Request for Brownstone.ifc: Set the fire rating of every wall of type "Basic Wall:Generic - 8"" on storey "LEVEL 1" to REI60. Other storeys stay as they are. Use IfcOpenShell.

First a look at what the model holds.

```python
import ifcopenshell
import ifcopenshell.util.element

model = ifcopenshell.open("Brownstone.ifc")
print(model.schema)
storey = next(s for s in model.by_type("IfcBuildingStorey") if s.Name == "LEVEL 1")
walls = [e for e in ifcopenshell.util.element.get_decomposition(storey) if e.is_a("IfcWall")]
seen = {}
for e in walls:
    element_type = ifcopenshell.util.element.get_type(e)
    key = (element_type.Name if element_type != e and element_type else None, ifcopenshell.util.element.get_pset(e, "Pset_WallCommon", "FireRating"))
    seen[key] = seen.get(key, 0) + 1
for (name, value), count in sorted(seen.items(), key=str):
    print(count, "x", name, "|", value)
```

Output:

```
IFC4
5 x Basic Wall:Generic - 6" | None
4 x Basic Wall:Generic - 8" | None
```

```python
import ifcopenshell
import ifcopenshell.api.pset
import ifcopenshell.util.element

model = ifcopenshell.open("Brownstone.ifc")

storey = next(s for s in model.by_type("IfcBuildingStorey") if s.Name == "LEVEL 1")
walls = [e for e in ifcopenshell.util.element.get_decomposition(storey) if e.is_a("IfcWall")]

count = 0
for e in walls:
    element_type = ifcopenshell.util.element.get_type(e)
    if element_type in (None, e) or element_type.Name != 'Basic Wall:Generic - 8"':
        continue
    # add_pset returns the element's existing set when there is one.
    pset = ifcopenshell.api.pset.add_pset(model, product=e, name="Pset_WallCommon")
    ifcopenshell.api.pset.edit_pset(model, pset=pset, properties={"FireRating": "REI60"})
    count += 1

print(count, "walls updated")

model.write("Brownstone-out.ifc")
```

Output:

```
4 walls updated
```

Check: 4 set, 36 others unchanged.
